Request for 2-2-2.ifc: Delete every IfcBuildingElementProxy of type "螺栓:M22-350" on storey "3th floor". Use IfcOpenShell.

First a look at what the model holds.

```python
import ifcopenshell
import ifcopenshell.util.element

model = ifcopenshell.open("2-2-2.ifc")
print(model.schema)
storey = next(s for s in model.by_type("IfcBuildingStorey") if s.Name == "3th floor")
proxies = [e for e in ifcopenshell.util.element.get_decomposition(storey) if e.is_a("IfcBuildingElementProxy")]
seen = {}
for e in proxies:
    element_type = ifcopenshell.util.element.get_type(e)
    name = element_type.Name if element_type not in (None, e) else None
    seen[name] = seen.get(name, 0) + 1
for name, count in sorted(seen.items(), key=str):
    print(count, "x", name)
```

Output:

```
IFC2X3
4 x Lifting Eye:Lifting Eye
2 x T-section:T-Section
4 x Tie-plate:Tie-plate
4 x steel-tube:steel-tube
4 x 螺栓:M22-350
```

```python
import ifcopenshell
import ifcopenshell.api.root
import ifcopenshell.util.element

model = ifcopenshell.open("2-2-2.ifc")

storey = next(s for s in model.by_type("IfcBuildingStorey") if s.Name == "3th floor")
proxies = [e for e in ifcopenshell.util.element.get_decomposition(storey) if e.is_a("IfcBuildingElementProxy")]
targets = [e for e in proxies if (t := ifcopenshell.util.element.get_type(e)) not in (None, e) and t.Name == "螺栓:M22-350"]

for e in targets:
    ifcopenshell.api.root.remove_product(model, product=e)
print(len(targets), "removed")

model.write("2-2-2_updated.ifc")
```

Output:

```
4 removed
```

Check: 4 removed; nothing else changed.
